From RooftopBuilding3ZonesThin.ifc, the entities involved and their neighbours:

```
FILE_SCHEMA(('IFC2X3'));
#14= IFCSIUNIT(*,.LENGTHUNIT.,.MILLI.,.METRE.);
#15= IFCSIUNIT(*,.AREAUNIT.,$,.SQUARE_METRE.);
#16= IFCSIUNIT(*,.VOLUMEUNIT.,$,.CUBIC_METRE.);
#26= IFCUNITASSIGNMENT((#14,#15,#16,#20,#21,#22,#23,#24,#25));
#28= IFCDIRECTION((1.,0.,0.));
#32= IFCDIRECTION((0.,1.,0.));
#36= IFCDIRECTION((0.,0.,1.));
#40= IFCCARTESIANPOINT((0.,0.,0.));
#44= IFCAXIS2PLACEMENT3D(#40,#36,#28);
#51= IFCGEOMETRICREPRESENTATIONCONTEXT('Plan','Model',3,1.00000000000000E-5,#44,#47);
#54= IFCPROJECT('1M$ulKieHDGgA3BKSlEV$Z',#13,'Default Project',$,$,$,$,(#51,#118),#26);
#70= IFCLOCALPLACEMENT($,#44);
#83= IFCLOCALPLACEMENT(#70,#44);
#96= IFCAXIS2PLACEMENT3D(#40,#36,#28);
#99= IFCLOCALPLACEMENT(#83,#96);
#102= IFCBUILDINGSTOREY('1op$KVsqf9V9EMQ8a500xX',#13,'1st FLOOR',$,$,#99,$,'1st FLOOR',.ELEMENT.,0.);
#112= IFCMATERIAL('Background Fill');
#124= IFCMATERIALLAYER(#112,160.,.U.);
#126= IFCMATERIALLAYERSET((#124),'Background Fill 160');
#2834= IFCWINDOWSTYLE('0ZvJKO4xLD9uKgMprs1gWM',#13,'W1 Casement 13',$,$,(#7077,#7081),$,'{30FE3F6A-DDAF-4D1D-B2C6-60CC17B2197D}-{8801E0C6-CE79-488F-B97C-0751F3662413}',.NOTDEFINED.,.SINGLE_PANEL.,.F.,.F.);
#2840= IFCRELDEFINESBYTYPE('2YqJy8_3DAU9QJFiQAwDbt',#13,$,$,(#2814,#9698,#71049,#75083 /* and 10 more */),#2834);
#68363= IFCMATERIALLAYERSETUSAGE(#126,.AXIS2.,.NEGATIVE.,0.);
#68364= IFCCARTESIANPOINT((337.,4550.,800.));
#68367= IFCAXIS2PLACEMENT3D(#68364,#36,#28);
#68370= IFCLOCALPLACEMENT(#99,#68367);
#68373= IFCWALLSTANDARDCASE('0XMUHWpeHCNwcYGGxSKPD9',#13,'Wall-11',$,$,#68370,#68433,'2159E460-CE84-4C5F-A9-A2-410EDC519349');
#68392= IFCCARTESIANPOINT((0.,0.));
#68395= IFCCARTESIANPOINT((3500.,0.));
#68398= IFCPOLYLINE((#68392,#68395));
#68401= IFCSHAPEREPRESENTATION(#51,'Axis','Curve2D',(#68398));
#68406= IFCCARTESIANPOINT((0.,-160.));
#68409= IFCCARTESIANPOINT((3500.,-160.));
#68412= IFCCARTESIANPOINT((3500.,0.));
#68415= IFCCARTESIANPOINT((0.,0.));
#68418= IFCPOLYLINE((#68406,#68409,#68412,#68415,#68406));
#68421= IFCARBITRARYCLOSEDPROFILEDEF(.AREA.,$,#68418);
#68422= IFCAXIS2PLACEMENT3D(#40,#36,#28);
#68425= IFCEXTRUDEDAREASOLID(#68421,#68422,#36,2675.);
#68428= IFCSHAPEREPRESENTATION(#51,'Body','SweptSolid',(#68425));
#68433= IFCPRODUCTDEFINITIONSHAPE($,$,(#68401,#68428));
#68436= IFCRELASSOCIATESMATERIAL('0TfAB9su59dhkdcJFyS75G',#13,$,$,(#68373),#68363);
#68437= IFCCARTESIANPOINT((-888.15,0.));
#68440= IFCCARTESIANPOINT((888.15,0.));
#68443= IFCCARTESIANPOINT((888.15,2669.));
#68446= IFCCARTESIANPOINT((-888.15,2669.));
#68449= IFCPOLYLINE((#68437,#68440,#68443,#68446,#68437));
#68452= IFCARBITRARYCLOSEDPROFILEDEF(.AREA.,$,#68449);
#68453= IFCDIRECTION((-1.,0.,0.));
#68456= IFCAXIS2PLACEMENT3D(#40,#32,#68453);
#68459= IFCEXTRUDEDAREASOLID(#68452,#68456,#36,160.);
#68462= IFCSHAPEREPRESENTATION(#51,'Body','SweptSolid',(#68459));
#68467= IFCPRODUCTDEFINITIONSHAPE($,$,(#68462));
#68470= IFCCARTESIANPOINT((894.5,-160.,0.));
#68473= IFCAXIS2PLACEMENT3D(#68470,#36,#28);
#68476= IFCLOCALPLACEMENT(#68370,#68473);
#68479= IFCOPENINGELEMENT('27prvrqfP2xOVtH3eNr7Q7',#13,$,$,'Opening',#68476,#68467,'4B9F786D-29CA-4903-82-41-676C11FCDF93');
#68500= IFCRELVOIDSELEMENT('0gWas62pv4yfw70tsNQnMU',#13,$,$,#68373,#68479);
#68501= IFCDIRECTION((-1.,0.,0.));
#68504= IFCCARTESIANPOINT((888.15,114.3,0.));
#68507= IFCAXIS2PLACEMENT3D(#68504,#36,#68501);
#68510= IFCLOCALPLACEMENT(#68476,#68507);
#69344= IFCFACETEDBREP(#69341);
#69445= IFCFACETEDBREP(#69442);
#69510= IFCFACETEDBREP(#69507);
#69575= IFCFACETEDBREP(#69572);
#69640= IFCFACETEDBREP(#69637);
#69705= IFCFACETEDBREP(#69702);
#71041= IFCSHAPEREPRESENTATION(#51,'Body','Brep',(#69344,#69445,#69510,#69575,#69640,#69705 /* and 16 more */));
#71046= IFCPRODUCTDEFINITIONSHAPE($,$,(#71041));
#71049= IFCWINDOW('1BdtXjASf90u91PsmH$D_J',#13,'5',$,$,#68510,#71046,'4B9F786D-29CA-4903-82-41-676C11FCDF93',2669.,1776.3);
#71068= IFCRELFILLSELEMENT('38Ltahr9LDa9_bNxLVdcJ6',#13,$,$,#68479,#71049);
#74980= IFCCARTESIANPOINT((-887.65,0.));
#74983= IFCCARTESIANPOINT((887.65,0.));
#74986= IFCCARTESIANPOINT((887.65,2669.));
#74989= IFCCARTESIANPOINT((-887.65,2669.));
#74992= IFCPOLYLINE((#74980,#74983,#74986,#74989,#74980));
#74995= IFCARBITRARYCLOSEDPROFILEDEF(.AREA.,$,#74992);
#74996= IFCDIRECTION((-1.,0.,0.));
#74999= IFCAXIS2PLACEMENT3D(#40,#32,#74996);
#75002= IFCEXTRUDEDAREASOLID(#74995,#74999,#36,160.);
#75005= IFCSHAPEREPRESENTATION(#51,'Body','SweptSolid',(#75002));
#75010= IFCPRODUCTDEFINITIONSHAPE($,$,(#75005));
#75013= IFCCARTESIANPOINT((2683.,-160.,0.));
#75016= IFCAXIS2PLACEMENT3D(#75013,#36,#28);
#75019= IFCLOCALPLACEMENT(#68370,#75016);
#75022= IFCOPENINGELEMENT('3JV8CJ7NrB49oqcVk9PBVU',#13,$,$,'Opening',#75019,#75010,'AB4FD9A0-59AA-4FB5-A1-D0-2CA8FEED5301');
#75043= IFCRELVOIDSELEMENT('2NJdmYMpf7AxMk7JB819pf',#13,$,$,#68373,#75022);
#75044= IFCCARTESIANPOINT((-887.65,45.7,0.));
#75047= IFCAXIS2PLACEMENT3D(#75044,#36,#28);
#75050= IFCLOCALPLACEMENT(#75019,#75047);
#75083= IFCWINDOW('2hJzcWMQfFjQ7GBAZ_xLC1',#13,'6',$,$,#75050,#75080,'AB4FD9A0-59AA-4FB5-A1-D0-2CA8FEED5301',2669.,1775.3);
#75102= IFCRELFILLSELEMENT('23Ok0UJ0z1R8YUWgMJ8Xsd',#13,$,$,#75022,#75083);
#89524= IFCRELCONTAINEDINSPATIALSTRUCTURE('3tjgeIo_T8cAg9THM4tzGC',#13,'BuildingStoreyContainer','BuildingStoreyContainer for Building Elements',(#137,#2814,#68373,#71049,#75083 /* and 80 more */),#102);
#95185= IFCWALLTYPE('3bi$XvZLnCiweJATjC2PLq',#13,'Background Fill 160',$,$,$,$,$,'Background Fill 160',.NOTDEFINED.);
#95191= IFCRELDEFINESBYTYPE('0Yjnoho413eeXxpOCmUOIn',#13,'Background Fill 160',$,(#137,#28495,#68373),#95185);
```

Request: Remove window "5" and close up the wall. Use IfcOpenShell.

```python
import ifcopenshell
import ifcopenshell.api.feature
import ifcopenshell.api.root
import ifcopenshell.geom
import ifcopenshell.util.shape

model = ifcopenshell.open("RooftopBuilding3ZonesThin.ifc")
settings = ifcopenshell.geom.settings()


def volume(element):
    """Net volume in cubic metres, openings subtracted."""
    shape = ifcopenshell.geom.create_shape(settings, element)
    return ifcopenshell.util.shape.get_volume(shape.geometry)


window = model.by_id(71049)
opening = window.FillsVoids[0].RelatingOpeningElement
wall = opening.VoidsElements[0].RelatingBuildingElement
before = volume(wall)

ifcopenshell.api.root.remove_product(model, product=window)
ifcopenshell.api.feature.remove_feature(model, feature=opening)

after = volume(wall)

print(f"wall volume {before:.3f} -> {after:.3f} m3")

model.write("RooftopBuilding3ZonesThin-out.ifc")
```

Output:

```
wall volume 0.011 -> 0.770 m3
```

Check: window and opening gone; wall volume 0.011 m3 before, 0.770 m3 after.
